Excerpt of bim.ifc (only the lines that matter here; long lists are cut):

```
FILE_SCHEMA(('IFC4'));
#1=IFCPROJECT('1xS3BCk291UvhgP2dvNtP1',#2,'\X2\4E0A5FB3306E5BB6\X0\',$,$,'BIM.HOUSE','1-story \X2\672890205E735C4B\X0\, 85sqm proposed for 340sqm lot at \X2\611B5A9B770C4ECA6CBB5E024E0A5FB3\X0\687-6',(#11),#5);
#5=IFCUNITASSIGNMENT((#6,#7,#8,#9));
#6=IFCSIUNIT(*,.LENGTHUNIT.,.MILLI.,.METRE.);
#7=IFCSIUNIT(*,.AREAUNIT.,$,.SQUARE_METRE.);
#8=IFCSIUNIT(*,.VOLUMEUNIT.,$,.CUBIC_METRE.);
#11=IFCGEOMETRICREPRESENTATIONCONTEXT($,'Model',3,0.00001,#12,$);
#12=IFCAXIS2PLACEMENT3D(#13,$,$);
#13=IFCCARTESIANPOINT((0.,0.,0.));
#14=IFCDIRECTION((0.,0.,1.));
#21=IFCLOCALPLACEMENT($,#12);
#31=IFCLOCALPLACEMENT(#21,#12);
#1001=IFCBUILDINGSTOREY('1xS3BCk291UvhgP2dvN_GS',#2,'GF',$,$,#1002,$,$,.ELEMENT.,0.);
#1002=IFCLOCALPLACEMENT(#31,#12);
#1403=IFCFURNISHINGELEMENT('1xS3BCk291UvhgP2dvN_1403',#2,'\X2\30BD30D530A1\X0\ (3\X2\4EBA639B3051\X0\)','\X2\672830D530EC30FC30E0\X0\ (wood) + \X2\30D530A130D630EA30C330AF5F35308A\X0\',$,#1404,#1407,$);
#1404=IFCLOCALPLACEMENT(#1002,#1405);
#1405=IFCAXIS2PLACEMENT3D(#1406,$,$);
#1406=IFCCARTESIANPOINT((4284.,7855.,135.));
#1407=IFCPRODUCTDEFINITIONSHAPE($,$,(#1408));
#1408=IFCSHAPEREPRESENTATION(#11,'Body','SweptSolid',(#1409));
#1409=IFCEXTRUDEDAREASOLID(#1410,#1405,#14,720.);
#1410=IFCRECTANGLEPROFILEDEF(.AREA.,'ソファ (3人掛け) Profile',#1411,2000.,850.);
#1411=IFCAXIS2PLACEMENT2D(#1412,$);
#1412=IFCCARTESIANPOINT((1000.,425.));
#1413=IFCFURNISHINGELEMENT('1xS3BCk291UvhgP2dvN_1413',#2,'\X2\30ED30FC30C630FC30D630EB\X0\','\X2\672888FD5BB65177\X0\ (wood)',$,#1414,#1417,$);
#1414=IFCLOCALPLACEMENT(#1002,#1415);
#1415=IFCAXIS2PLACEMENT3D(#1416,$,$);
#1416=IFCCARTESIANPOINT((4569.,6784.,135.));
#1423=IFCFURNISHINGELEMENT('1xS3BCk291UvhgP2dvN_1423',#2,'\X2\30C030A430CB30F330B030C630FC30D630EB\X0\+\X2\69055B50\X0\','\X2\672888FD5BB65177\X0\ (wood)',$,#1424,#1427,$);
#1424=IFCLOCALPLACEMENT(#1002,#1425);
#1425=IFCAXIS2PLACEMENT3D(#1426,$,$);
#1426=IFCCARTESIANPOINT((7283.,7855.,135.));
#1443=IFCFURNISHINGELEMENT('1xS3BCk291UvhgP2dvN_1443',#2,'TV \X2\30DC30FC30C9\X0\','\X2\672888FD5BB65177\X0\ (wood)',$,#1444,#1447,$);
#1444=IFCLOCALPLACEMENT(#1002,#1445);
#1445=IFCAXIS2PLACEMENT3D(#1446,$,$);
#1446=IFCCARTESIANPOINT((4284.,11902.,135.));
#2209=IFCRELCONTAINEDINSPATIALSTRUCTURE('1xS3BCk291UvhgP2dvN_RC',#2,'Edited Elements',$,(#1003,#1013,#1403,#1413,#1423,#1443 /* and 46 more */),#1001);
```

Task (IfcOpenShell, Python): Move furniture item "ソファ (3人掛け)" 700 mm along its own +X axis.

```python
import ifcopenshell
import ifcopenshell.api.geometry
import ifcopenshell.util.placement

model = ifcopenshell.open("bim.ifc")

item = model.by_id(1403)
matrix = ifcopenshell.util.placement.get_local_placement(item.ObjectPlacement)
matrix[:3, 3] += matrix[:3, 0] * 700.0
ifcopenshell.api.geometry.edit_object_placement(model, product=item, matrix=matrix, is_si=False)

print(ifcopenshell.util.placement.get_local_placement(item.ObjectPlacement).round(3) + 0.0)

model.write("bim_v2.ifc")
```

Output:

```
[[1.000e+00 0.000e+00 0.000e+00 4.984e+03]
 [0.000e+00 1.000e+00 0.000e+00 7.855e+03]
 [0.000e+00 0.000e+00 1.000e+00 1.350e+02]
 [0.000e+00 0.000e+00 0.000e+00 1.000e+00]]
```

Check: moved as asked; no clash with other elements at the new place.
